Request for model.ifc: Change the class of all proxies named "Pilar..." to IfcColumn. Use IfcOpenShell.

First a look at what the model holds.

```python
import re

import ifcopenshell

model = ifcopenshell.open("model.ifc")
print(model.schema)
seen = {}
for e in model.by_type("IfcBuildingElementProxy"):
    name = re.sub(r":\d+(:\d+)?$", "", e.Name or "")  # drop the element id that some exporters append
    seen[name] = seen.get(name, 0) + 1
for name, count in sorted(seen.items()):
    print(count, "x", name)
```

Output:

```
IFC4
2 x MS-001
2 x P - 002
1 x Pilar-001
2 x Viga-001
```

```python
import ifcopenshell
import ifcopenshell.api.root

model = ifcopenshell.open("model.ifc")

proxies = [e.id() for e in model.by_type("IfcBuildingElementProxy") if (e.Name or "").startswith("Pilar")]
for step_id in proxies:
    proxy = model.by_id(step_id)
    # Reclassifying a typed element also reclassifies its type and the type's other occurrences.
    if proxy.is_a("IfcBuildingElementProxy"):
        ifcopenshell.api.root.reassign_class(model, product=proxy, ifc_class="IfcColumn")

print(sum(model.by_id(i).is_a("IfcColumn") for i in proxies), "reclassified")

model.write("model_rev.ifc")
```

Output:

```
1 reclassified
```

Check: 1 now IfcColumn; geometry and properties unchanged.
